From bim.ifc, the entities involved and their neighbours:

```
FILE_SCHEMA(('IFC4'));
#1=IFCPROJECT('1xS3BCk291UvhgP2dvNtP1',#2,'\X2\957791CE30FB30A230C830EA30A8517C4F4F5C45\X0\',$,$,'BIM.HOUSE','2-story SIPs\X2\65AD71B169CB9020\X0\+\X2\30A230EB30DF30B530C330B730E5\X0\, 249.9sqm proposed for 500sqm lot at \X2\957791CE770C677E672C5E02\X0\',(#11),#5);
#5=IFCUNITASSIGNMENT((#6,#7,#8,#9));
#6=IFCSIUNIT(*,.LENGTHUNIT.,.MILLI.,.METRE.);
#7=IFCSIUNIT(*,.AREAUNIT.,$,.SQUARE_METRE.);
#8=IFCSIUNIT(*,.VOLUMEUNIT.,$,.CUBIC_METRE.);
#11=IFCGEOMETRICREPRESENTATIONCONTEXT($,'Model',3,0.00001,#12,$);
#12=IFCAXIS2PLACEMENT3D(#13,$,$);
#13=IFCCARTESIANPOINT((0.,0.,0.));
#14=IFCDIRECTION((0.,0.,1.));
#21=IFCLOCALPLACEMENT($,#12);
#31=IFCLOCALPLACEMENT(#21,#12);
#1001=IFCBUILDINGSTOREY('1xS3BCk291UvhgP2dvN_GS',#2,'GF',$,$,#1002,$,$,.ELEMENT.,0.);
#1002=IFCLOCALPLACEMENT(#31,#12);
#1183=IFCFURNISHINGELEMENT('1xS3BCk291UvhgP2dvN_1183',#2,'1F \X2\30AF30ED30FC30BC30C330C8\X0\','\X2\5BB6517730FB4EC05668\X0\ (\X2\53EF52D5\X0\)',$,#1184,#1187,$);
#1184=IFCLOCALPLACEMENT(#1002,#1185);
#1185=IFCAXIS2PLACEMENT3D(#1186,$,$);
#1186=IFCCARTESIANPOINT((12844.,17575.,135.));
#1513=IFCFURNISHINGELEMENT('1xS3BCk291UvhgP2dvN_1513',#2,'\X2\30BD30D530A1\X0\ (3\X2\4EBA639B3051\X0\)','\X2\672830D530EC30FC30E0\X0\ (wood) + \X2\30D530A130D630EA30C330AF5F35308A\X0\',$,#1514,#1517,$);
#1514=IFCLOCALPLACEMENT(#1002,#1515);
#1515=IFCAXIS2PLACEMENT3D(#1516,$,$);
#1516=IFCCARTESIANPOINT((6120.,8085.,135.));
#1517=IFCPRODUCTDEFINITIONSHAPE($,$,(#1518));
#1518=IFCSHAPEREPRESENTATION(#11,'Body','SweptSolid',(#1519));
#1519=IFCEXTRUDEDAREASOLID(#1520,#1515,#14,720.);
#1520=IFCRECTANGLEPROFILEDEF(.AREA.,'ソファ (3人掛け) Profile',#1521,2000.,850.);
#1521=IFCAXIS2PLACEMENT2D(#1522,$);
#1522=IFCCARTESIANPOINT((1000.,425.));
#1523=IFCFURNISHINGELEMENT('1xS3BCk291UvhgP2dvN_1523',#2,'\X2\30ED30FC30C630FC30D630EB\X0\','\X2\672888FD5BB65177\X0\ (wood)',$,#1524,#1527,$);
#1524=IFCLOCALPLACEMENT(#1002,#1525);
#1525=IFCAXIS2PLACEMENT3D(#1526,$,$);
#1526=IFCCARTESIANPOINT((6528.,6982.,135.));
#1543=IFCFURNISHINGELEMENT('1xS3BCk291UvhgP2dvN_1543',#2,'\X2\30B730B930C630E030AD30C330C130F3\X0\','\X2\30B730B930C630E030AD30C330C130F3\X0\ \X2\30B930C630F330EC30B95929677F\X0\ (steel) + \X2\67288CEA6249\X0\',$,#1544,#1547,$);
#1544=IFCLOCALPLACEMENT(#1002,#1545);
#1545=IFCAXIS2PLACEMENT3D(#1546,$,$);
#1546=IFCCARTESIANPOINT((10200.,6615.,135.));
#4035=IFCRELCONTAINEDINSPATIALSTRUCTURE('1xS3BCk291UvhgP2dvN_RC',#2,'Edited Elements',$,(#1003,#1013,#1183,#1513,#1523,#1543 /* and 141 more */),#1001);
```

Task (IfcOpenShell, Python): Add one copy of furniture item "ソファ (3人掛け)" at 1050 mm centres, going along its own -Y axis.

```python
import ifcopenshell
import ifcopenshell.api.geometry
import ifcopenshell.api.root
import ifcopenshell.util.element
import ifcopenshell.util.placement
import ifcopenshell.util.unit

model = ifcopenshell.open("bim.ifc")
unit_scale = ifcopenshell.util.unit.calculate_unit_scale(model)


def reuse_history(source, copy):
    """copy_class also copies each property set's owner history, people and application; keep the originals."""
    for rel in copy.IsDefinedBy:
        if rel.is_a("IfcRelDefinesByProperties") and (history := rel.RelatingPropertyDefinition.OwnerHistory):
            rel.RelatingPropertyDefinition.OwnerHistory = source.OwnerHistory
            ifcopenshell.util.element.remove_deep2(model, history)


source = model.by_guid("1xS3BCk291UvhgP2dvN_1513")
base = ifcopenshell.util.placement.get_local_placement(source.ObjectPlacement)
step = -base[:3, 1] * 1.05 / unit_scale

for i in range(1, 2):
    copy = ifcopenshell.api.root.copy_class(model, product=source)
    copy.Representation = ifcopenshell.util.element.copy_deep(
        model, source.Representation, exclude=["IfcGeometricRepresentationContext", "IfcRepresentationMap"]
    )
    reuse_history(source, copy)
    matrix = base.copy()
    matrix[:3, 3] += i * step
    print("added at", matrix[:3, 3].round(3) + 0.0)
    ifcopenshell.api.geometry.edit_object_placement(model, product=copy, matrix=matrix, is_si=False)

model.write("bim_v2.ifc")
```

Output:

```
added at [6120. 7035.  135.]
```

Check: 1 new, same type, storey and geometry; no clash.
